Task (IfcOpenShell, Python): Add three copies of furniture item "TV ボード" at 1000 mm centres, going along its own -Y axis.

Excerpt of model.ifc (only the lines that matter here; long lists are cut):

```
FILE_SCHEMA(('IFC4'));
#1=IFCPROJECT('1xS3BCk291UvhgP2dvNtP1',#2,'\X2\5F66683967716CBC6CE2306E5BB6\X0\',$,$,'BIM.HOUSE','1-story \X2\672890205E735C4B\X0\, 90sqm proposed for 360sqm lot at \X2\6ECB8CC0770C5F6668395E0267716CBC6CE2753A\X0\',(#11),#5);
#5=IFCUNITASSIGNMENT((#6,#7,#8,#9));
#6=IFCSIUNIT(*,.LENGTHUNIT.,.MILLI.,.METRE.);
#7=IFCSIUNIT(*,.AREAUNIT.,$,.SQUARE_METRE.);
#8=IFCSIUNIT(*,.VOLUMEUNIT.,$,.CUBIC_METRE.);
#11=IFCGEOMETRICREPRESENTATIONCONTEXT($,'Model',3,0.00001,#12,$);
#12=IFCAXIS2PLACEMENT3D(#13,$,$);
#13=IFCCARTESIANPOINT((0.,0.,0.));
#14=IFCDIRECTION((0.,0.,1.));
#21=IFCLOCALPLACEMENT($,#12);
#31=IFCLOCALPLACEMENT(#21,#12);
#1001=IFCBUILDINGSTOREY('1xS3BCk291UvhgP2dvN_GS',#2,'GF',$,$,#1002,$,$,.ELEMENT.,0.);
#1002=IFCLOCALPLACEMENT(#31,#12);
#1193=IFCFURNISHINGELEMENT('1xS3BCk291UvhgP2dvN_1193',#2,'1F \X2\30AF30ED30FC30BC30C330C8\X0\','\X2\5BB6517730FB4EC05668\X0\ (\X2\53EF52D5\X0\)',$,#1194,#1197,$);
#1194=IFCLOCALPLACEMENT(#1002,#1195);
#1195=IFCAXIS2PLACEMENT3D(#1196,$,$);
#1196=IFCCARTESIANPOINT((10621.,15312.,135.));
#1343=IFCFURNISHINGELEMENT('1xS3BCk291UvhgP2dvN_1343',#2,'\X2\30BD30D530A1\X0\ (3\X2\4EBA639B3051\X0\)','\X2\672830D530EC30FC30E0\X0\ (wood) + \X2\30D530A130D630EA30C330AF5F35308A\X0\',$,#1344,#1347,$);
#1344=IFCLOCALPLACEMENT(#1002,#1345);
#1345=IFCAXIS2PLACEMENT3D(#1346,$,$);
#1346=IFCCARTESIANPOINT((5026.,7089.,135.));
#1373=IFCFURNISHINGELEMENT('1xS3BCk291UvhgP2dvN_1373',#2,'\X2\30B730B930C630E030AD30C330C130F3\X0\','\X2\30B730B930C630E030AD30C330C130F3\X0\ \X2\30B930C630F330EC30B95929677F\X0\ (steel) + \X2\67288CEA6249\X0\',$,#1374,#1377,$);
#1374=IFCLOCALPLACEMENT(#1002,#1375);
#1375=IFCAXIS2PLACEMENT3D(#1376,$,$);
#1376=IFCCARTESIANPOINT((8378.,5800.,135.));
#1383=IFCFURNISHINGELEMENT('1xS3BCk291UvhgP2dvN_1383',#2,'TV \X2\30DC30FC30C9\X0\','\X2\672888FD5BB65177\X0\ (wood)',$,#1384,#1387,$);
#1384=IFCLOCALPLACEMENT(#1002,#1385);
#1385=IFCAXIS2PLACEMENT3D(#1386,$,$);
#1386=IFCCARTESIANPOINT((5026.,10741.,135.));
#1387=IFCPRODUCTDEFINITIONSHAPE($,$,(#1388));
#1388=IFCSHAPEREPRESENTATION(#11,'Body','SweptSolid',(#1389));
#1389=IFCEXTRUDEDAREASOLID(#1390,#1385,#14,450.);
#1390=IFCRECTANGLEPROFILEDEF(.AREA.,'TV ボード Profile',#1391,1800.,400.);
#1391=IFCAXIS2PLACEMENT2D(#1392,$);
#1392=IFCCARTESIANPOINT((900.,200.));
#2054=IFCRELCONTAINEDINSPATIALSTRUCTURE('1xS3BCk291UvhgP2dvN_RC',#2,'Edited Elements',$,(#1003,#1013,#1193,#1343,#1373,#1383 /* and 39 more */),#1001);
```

```python
import ifcopenshell
import ifcopenshell.api.geometry
import ifcopenshell.api.root
import ifcopenshell.util.element
import ifcopenshell.util.placement

model = ifcopenshell.open("model.ifc")


def reuse_history(source, copy):
    """copy_class also copies each property set's owner history, people and application; keep the originals."""
    for rel in copy.IsDefinedBy:
        if rel.is_a("IfcRelDefinesByProperties") and (history := rel.RelatingPropertyDefinition.OwnerHistory):
            rel.RelatingPropertyDefinition.OwnerHistory = source.OwnerHistory
            ifcopenshell.util.element.remove_deep2(model, history)


source = model.by_guid("1xS3BCk291UvhgP2dvN_1383")
base = ifcopenshell.util.placement.get_local_placement(source.ObjectPlacement)
step = -base[:3, 1] * 1000.0

for i in range(1, 4):
    copy = ifcopenshell.api.root.copy_class(model, product=source)
    copy.Representation = ifcopenshell.util.element.copy_deep(
        model, source.Representation, exclude=["IfcGeometricRepresentationContext", "IfcRepresentationMap"]
    )
    reuse_history(source, copy)
    matrix = base.copy()
    matrix[:3, 3] += i * step
    print("added at", matrix[:3, 3].round(3) + 0.0)
    ifcopenshell.api.geometry.edit_object_placement(model, product=copy, matrix=matrix, is_si=False)

model.write("model_v2.ifc")
```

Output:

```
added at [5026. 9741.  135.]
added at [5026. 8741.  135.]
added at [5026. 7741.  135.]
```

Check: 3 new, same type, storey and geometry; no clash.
